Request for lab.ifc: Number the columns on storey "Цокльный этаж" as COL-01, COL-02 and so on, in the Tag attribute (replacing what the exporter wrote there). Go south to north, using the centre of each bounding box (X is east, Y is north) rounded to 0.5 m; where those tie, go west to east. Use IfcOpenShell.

First a look at what the model holds.

```python
import ifcopenshell
import ifcopenshell.util.element
import ifcopenshell.util.placement

model = ifcopenshell.open("lab.ifc")
print(model.schema)
storey = next(s for s in model.by_type("IfcBuildingStorey") if s.Name == "Цокльный этаж")
columns = [e for e in ifcopenshell.util.element.get_decomposition(storey) if e.is_a("IfcColumn")]
for e in sorted(columns, key=lambda e: e.id()):
    origin = ifcopenshell.util.placement.get_local_placement(e.ObjectPlacement)[:3, 3]
    print(e.id(), e.Tag, e.Name, origin.round(2) + 0.0, sep=" | ")
```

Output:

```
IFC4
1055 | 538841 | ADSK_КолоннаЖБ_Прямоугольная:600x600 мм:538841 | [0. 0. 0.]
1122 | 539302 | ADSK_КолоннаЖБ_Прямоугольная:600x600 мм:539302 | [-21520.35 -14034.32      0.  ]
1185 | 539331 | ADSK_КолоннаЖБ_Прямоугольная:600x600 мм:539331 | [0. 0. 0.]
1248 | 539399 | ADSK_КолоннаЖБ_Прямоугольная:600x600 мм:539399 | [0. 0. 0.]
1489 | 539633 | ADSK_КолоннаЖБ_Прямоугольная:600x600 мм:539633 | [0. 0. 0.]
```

```python
import ifcopenshell
import ifcopenshell.geom
import ifcopenshell.util.element
import ifcopenshell.util.shape

model = ifcopenshell.open("lab.ifc")
settings = ifcopenshell.geom.settings()
settings.set("use-world-coords", True)


def centre(element):
    shape = ifcopenshell.geom.create_shape(settings, element)
    return ifcopenshell.util.shape.get_bbox_centroid(shape.geometry)


storey = next(s for s in model.by_type("IfcBuildingStorey") if s.Name == "Цокльный этаж")
columns = [e for e in ifcopenshell.util.element.get_decomposition(storey) if e.is_a("IfcColumn")]

# Insertion points can sit at a corner or the storey origin, so sort by the geometry (in metres).
centres = {e: centre(e) for e in columns}
columns.sort(key=lambda e: (round(centres[e][1] / 0.5), centres[e][0]))

for i, e in enumerate(columns, start=1):
    number = f"COL-{i:02d}"
    e.Tag = number
    print(e.id(), number)

model.write("lab_rev.ifc")
```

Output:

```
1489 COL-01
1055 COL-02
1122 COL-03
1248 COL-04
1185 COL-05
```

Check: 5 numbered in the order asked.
